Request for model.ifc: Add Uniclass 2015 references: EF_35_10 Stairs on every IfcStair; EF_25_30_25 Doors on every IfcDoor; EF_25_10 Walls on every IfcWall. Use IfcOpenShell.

First a look at what the model holds.

```python
import ifcopenshell

model = ifcopenshell.open("model.ifc")
print(model.schema)
print("classifications:", [c.Name for c in model.by_type("IfcClassification")])
for ifc_class in ("IfcDoor", "IfcRoof", "IfcStair", "IfcWall", "IfcWindow"):
    print(ifc_class, len(model.by_type(ifc_class)))
```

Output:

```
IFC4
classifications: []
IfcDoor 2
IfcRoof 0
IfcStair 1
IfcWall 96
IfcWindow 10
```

```python
import ifcopenshell
import ifcopenshell.api.classification

model = ifcopenshell.open("model.ifc")

system = ifcopenshell.api.classification.add_classification(model, classification="Uniclass 2015")

codes = {
    "IfcStair": ("EF_35_10", "Stairs"),
    "IfcDoor": ("EF_25_30_25", "Doors"),
    "IfcWall": ("EF_25_10", "Walls"),
}
for ifc_class, (code, name) in codes.items():
    products = model.by_type(ifc_class)
    ifcopenshell.api.classification.add_reference(
        model, products=products, classification=system, identification=code, name=name
    )
    print(code, len(products))

model.write("model_rev.ifc")
```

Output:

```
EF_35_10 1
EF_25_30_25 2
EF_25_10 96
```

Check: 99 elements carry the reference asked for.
